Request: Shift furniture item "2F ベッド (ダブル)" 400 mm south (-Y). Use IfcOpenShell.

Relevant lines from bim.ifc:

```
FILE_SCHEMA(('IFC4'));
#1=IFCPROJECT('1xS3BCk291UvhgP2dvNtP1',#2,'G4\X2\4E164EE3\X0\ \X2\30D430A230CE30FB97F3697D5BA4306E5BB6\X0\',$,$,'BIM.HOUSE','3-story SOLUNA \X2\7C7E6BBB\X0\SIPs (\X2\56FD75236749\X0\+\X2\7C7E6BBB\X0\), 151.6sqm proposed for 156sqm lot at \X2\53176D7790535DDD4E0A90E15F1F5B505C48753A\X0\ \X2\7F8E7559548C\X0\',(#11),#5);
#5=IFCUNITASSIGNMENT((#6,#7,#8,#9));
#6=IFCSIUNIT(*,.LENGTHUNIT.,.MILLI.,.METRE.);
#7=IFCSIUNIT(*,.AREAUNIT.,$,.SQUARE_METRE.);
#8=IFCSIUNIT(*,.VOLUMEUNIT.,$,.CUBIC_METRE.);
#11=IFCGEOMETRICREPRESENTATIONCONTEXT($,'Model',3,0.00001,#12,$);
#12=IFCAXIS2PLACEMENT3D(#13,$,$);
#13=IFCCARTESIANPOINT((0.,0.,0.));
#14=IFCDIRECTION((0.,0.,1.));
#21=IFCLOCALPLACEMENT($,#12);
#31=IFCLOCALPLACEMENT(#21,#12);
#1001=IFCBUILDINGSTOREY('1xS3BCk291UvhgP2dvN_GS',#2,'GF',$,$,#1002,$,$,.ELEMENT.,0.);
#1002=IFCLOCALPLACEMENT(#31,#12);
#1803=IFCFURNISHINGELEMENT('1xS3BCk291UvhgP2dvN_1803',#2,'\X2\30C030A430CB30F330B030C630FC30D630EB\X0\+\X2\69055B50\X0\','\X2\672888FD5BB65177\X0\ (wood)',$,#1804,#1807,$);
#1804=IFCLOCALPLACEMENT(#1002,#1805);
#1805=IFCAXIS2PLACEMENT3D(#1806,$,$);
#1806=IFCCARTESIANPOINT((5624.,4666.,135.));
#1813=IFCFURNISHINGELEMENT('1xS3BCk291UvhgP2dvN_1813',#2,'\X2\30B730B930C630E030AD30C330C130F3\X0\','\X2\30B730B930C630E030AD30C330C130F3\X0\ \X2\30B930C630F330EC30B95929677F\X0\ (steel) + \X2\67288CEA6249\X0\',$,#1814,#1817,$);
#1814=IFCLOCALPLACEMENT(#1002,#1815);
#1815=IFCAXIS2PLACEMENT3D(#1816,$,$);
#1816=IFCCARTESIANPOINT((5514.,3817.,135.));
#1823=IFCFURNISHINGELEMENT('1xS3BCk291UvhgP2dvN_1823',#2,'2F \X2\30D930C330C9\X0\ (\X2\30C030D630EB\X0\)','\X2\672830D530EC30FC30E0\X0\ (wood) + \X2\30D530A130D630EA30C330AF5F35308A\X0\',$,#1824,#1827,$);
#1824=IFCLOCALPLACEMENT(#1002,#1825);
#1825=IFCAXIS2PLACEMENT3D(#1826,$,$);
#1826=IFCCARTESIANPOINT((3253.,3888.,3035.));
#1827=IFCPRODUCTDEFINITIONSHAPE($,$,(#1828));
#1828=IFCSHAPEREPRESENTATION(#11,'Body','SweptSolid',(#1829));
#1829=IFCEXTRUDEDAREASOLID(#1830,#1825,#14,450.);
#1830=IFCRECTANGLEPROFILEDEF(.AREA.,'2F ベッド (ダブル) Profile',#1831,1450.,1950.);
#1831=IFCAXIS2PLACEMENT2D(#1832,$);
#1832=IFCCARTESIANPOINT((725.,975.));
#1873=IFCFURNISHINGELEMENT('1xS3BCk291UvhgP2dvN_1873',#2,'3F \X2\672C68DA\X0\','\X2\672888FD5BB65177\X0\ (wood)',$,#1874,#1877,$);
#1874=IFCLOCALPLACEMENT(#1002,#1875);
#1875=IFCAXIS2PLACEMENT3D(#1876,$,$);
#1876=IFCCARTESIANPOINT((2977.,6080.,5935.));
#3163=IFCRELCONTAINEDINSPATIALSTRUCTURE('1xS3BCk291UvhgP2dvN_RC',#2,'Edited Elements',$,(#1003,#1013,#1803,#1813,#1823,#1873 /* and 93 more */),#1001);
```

```python
import ifcopenshell
import ifcopenshell.api.geometry
import ifcopenshell.util.placement

model = ifcopenshell.open("bim.ifc")

item = model.by_guid("1xS3BCk291UvhgP2dvN_1823")
matrix = ifcopenshell.util.placement.get_local_placement(item.ObjectPlacement)
matrix[1, 3] -= 400.0
ifcopenshell.api.geometry.edit_object_placement(model, product=item, matrix=matrix, is_si=False)

print(ifcopenshell.util.placement.get_local_placement(item.ObjectPlacement).round(3) + 0.0)

model.write("bim_edited.ifc")
```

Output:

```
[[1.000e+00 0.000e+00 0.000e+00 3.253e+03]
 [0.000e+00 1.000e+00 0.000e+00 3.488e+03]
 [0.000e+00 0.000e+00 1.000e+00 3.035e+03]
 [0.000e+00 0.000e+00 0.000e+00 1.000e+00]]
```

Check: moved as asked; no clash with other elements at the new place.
